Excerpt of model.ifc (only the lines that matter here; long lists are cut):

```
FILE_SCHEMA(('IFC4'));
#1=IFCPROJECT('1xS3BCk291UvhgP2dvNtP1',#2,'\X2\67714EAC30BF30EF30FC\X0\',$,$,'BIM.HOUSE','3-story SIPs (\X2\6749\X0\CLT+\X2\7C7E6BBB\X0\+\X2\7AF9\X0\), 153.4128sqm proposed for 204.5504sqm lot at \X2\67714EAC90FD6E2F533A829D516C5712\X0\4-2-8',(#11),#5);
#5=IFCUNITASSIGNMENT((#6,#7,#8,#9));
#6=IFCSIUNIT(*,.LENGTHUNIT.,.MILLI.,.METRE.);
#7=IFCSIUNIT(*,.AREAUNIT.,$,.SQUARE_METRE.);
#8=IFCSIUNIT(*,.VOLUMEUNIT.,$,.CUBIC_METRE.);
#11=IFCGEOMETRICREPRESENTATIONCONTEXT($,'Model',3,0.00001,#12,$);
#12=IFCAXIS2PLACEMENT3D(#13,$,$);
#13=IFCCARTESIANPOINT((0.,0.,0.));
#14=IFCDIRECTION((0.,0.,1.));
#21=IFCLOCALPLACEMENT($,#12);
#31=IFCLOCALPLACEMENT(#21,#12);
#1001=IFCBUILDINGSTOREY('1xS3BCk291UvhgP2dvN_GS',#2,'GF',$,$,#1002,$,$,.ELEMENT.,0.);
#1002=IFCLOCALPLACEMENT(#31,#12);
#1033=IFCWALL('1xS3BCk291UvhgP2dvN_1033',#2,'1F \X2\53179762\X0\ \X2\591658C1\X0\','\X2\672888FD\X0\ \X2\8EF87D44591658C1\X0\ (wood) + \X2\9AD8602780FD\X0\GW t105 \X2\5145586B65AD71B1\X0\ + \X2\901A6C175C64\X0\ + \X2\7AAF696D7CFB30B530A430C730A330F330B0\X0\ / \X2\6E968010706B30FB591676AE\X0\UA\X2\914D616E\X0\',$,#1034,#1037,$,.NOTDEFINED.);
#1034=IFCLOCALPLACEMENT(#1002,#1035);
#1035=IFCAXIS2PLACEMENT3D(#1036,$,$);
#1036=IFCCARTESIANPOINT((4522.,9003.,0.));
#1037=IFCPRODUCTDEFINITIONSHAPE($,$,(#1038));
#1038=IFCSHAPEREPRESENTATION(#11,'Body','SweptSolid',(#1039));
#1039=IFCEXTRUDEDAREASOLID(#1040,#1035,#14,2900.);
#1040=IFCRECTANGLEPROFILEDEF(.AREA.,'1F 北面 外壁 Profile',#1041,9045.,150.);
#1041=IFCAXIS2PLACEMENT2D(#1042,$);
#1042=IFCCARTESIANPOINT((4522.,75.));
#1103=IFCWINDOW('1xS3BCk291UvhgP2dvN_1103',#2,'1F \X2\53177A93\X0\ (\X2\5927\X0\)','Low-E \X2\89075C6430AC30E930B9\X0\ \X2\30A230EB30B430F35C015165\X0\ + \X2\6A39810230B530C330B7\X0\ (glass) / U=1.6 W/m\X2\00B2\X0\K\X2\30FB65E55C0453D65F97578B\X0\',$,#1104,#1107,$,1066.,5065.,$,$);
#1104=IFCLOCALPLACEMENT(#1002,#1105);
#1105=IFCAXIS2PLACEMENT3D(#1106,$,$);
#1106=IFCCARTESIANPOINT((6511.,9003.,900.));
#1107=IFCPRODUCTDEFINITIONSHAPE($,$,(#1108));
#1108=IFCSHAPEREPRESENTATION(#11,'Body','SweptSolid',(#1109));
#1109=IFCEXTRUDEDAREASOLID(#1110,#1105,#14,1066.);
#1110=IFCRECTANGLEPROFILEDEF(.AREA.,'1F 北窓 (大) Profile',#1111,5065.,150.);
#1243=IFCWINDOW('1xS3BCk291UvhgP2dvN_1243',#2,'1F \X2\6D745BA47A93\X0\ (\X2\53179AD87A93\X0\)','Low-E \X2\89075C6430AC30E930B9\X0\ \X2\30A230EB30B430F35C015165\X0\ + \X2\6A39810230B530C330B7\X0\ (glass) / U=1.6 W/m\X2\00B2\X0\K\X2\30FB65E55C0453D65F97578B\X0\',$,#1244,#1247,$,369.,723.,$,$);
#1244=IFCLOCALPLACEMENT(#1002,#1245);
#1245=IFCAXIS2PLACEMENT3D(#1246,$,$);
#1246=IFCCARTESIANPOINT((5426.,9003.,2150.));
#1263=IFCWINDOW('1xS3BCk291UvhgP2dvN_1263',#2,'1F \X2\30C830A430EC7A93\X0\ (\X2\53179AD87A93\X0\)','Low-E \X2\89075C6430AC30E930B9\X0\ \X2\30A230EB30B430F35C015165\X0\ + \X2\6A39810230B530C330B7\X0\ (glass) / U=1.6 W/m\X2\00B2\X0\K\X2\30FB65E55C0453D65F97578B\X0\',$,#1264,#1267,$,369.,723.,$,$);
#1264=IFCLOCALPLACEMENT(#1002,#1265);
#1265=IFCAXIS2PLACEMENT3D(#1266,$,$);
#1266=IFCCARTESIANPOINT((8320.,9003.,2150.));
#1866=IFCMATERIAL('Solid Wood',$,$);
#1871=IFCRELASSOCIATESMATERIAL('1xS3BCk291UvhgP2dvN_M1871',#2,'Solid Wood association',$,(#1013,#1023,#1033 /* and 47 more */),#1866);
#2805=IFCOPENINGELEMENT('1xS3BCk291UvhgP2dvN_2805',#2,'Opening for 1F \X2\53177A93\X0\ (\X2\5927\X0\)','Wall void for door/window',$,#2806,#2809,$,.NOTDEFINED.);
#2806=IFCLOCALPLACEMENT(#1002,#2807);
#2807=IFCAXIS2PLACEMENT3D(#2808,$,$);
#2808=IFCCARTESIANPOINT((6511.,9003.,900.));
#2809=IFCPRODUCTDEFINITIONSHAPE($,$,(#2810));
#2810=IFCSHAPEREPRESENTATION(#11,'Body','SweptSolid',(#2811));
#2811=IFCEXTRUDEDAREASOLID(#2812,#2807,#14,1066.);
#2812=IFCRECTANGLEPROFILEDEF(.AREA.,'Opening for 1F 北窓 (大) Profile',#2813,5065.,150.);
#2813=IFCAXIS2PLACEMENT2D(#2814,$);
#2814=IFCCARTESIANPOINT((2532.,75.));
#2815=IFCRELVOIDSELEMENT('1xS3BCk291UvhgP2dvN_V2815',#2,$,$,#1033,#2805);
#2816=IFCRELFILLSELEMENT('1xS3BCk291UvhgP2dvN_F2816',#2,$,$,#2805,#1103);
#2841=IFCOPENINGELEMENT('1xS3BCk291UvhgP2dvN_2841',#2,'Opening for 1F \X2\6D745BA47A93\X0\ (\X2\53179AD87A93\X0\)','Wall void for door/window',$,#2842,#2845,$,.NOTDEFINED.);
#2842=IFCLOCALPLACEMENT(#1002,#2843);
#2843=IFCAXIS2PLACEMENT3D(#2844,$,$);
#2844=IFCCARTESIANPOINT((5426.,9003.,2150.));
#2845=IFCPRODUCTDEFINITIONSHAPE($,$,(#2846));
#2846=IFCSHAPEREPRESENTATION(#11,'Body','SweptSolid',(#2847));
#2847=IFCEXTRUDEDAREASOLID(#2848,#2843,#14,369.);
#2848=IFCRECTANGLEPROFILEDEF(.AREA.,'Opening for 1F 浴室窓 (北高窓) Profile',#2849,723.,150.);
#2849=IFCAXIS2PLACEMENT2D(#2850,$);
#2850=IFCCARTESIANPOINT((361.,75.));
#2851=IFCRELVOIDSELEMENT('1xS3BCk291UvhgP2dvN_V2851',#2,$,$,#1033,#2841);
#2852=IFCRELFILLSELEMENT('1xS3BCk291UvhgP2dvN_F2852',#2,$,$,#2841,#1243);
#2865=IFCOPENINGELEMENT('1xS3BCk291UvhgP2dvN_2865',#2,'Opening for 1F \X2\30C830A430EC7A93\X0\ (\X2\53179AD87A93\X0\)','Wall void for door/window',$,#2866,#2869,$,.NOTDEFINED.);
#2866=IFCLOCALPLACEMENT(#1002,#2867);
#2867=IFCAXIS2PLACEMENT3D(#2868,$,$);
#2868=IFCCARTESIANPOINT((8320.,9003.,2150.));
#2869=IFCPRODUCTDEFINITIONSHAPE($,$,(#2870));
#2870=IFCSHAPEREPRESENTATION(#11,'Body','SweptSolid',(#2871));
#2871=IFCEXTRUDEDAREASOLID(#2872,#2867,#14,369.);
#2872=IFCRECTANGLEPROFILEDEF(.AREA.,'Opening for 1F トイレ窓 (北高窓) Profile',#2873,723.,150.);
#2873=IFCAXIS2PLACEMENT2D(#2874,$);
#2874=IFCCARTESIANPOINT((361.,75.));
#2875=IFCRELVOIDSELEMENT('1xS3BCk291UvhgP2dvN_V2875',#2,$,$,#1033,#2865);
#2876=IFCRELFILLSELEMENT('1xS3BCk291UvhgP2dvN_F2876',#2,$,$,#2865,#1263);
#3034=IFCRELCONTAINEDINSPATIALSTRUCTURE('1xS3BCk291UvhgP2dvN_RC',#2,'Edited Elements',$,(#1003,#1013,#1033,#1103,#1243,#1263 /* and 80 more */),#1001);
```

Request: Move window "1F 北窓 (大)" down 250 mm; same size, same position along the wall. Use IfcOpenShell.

```python
import numpy as np
import ifcopenshell
import ifcopenshell.api.geometry
import ifcopenshell.util.placement
import ifcopenshell.util.unit

model = ifcopenshell.open("model.ifc")
unit_scale = ifcopenshell.util.unit.calculate_unit_scale(model)

window = model.by_id(1103)
opening = window.FillsVoids[0].RelatingOpeningElement
dz = -0.25 / unit_scale

shift = np.array([0.0, 0.0, dz])
# The window is not placed relative to its opening, so move both.
for product in (opening, window):
    matrix = ifcopenshell.util.placement.get_local_placement(product.ObjectPlacement)
    matrix[:3, 3] += shift
    ifcopenshell.api.geometry.edit_object_placement(model, product=product, matrix=matrix, is_si=False)

print(f"moved by {dz * unit_scale:+.3f} m")

model.write("model_updated.ifc")
```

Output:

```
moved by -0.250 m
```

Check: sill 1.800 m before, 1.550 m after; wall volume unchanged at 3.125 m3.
